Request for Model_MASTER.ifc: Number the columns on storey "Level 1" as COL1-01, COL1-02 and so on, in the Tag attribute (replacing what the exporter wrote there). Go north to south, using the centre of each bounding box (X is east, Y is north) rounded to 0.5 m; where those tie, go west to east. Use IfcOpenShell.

First a look at what the model holds.

```python
import ifcopenshell
import ifcopenshell.util.element
import ifcopenshell.util.placement

model = ifcopenshell.open("Model_MASTER.ifc")
print(model.schema)
storey = next(s for s in model.by_type("IfcBuildingStorey") if s.Name == "Level 1")
columns = [e for e in ifcopenshell.util.element.get_decomposition(storey) if e.is_a("IfcColumn")]
for e in sorted(columns, key=lambda e: e.id()):
    origin = ifcopenshell.util.placement.get_local_placement(e.ObjectPlacement)[:3, 3]
    print(e.id(), e.Tag, e.Name, origin.round(2) + 0.0, sep=" | ")
```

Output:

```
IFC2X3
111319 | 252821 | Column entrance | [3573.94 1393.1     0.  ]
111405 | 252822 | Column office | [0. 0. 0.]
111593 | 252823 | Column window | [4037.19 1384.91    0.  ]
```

```python
import ifcopenshell
import ifcopenshell.geom
import ifcopenshell.util.element
import ifcopenshell.util.shape

model = ifcopenshell.open("Model_MASTER.ifc")
settings = ifcopenshell.geom.settings()
settings.set("use-world-coords", True)


def centre(element):
    shape = ifcopenshell.geom.create_shape(settings, element)
    return ifcopenshell.util.shape.get_bbox_centroid(shape.geometry)


storey = next(s for s in model.by_type("IfcBuildingStorey") if s.Name == "Level 1")
columns = [e for e in ifcopenshell.util.element.get_decomposition(storey) if e.is_a("IfcColumn")]

# Insertion points can sit at a corner or the storey origin, so sort by the geometry (in metres).
centres = {e: centre(e) for e in columns}
columns.sort(key=lambda e: (-round(centres[e][1] / 0.5), centres[e][0]))

for i, e in enumerate(columns, start=1):
    number = f"COL1-{i:02d}"
    e.Tag = number
    print(e.id(), number)

model.write("Model_MASTER_edited.ifc")
```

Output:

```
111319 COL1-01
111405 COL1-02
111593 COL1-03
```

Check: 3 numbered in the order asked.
